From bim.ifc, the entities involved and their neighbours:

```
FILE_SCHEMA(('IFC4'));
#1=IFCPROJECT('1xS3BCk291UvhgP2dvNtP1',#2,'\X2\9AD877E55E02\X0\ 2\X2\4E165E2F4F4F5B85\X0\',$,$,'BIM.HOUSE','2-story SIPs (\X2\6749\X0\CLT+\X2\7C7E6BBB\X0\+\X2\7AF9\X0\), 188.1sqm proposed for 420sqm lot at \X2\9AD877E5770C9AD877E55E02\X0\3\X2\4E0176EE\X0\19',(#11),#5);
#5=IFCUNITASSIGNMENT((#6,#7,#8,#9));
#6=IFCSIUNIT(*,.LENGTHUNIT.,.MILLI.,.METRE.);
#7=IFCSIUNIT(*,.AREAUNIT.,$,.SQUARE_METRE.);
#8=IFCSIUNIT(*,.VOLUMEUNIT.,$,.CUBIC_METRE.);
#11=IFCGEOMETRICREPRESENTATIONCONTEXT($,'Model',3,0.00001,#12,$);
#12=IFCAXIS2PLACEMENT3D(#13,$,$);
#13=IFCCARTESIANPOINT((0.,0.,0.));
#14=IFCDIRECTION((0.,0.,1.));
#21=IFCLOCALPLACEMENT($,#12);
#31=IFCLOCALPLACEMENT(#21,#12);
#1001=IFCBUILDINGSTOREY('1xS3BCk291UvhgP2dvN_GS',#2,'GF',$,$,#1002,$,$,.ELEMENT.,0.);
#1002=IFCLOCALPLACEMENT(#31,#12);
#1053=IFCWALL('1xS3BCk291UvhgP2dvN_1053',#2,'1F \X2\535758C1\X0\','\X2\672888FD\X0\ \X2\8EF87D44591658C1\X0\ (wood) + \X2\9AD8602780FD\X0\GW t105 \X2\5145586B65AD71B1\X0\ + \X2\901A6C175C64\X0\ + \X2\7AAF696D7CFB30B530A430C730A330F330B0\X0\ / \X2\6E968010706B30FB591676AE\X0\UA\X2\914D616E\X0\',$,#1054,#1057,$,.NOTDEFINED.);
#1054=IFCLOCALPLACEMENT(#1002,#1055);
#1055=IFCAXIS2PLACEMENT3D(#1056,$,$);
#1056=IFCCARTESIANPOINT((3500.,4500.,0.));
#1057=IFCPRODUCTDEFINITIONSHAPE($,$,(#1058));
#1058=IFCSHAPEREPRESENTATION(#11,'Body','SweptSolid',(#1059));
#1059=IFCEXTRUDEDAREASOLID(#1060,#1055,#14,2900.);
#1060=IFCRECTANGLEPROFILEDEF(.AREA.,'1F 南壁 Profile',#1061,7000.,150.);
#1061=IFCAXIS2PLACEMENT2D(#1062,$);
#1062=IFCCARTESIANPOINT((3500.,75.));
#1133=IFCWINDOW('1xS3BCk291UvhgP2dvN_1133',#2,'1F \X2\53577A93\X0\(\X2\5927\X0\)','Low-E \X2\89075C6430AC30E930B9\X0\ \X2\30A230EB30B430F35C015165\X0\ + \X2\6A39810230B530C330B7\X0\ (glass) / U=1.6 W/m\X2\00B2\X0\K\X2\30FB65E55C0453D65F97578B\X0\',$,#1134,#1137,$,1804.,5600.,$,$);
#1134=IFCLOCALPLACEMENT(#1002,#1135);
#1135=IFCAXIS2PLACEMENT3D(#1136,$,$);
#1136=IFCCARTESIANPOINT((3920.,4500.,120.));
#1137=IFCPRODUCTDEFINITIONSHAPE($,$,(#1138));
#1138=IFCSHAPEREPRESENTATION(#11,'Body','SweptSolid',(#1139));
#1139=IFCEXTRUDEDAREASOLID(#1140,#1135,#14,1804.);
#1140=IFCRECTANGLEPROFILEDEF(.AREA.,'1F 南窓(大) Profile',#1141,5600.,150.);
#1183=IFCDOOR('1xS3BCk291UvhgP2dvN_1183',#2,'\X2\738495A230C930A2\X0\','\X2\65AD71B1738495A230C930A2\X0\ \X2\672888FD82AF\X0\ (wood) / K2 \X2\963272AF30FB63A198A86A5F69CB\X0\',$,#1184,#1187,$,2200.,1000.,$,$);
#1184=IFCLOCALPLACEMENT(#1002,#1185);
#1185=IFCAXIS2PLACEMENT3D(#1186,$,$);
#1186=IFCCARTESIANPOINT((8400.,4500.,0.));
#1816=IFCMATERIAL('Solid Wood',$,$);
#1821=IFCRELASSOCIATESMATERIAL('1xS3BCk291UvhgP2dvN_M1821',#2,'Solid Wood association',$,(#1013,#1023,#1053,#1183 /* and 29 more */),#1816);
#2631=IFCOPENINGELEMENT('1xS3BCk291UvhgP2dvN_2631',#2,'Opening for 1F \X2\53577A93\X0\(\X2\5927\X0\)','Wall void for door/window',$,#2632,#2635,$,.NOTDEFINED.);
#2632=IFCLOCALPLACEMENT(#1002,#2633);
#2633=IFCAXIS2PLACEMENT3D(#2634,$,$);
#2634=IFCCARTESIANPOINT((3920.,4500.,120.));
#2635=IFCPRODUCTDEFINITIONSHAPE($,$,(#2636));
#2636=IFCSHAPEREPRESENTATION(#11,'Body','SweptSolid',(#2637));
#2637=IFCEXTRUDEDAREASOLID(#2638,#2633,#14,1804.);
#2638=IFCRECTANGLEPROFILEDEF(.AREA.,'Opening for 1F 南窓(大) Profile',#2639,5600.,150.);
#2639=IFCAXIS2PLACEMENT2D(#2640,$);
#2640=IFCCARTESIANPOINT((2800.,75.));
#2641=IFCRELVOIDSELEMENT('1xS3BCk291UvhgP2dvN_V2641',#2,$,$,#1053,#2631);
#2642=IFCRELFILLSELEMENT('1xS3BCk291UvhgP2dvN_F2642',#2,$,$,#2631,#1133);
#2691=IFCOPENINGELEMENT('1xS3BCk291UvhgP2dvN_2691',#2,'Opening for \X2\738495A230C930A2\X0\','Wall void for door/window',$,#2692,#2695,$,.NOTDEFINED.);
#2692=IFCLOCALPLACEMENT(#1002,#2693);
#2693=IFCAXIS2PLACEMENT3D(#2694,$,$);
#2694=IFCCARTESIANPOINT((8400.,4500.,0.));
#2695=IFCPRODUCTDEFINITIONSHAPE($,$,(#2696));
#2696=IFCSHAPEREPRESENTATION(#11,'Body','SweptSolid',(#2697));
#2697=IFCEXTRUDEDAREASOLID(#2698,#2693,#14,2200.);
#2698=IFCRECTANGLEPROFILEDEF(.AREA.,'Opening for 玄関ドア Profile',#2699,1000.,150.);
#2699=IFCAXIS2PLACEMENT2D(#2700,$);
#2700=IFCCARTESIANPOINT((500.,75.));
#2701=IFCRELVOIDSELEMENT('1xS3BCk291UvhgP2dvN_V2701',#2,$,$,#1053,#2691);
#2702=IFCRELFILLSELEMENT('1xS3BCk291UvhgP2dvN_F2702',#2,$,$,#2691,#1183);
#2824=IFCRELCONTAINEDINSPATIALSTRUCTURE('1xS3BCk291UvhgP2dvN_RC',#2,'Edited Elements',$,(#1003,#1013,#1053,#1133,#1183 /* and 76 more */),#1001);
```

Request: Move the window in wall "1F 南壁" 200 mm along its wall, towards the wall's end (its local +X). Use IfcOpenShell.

```python
import ifcopenshell
import ifcopenshell.api.geometry
import ifcopenshell.util.placement
import ifcopenshell.util.unit

model = ifcopenshell.open("bim.ifc")
unit_scale = ifcopenshell.util.unit.calculate_unit_scale(model)

window = model.by_guid("1xS3BCk291UvhgP2dvN_1133")
opening = window.FillsVoids[0].RelatingOpeningElement
wall = opening.VoidsElements[0].RelatingBuildingElement

wall_matrix = ifcopenshell.util.placement.get_local_placement(wall.ObjectPlacement)
shift = wall_matrix[:3, 0] * 0.2 / unit_scale
before = ifcopenshell.util.placement.get_local_placement(window.ObjectPlacement)[:3, 3].copy()

# The window is not placed relative to its opening, so move both.
for product in (opening, window):
    matrix = ifcopenshell.util.placement.get_local_placement(product.ObjectPlacement)
    matrix[:3, 3] += shift
    ifcopenshell.api.geometry.edit_object_placement(model, product=product, matrix=matrix, is_si=False)

after = ifcopenshell.util.placement.get_local_placement(window.ObjectPlacement)[:3, 3]
print("window moved by", (after - before).round(3) + 0.0)

model.write("bim_v2.ifc")
```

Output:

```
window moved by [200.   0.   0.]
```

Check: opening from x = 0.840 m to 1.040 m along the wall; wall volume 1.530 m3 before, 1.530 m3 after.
